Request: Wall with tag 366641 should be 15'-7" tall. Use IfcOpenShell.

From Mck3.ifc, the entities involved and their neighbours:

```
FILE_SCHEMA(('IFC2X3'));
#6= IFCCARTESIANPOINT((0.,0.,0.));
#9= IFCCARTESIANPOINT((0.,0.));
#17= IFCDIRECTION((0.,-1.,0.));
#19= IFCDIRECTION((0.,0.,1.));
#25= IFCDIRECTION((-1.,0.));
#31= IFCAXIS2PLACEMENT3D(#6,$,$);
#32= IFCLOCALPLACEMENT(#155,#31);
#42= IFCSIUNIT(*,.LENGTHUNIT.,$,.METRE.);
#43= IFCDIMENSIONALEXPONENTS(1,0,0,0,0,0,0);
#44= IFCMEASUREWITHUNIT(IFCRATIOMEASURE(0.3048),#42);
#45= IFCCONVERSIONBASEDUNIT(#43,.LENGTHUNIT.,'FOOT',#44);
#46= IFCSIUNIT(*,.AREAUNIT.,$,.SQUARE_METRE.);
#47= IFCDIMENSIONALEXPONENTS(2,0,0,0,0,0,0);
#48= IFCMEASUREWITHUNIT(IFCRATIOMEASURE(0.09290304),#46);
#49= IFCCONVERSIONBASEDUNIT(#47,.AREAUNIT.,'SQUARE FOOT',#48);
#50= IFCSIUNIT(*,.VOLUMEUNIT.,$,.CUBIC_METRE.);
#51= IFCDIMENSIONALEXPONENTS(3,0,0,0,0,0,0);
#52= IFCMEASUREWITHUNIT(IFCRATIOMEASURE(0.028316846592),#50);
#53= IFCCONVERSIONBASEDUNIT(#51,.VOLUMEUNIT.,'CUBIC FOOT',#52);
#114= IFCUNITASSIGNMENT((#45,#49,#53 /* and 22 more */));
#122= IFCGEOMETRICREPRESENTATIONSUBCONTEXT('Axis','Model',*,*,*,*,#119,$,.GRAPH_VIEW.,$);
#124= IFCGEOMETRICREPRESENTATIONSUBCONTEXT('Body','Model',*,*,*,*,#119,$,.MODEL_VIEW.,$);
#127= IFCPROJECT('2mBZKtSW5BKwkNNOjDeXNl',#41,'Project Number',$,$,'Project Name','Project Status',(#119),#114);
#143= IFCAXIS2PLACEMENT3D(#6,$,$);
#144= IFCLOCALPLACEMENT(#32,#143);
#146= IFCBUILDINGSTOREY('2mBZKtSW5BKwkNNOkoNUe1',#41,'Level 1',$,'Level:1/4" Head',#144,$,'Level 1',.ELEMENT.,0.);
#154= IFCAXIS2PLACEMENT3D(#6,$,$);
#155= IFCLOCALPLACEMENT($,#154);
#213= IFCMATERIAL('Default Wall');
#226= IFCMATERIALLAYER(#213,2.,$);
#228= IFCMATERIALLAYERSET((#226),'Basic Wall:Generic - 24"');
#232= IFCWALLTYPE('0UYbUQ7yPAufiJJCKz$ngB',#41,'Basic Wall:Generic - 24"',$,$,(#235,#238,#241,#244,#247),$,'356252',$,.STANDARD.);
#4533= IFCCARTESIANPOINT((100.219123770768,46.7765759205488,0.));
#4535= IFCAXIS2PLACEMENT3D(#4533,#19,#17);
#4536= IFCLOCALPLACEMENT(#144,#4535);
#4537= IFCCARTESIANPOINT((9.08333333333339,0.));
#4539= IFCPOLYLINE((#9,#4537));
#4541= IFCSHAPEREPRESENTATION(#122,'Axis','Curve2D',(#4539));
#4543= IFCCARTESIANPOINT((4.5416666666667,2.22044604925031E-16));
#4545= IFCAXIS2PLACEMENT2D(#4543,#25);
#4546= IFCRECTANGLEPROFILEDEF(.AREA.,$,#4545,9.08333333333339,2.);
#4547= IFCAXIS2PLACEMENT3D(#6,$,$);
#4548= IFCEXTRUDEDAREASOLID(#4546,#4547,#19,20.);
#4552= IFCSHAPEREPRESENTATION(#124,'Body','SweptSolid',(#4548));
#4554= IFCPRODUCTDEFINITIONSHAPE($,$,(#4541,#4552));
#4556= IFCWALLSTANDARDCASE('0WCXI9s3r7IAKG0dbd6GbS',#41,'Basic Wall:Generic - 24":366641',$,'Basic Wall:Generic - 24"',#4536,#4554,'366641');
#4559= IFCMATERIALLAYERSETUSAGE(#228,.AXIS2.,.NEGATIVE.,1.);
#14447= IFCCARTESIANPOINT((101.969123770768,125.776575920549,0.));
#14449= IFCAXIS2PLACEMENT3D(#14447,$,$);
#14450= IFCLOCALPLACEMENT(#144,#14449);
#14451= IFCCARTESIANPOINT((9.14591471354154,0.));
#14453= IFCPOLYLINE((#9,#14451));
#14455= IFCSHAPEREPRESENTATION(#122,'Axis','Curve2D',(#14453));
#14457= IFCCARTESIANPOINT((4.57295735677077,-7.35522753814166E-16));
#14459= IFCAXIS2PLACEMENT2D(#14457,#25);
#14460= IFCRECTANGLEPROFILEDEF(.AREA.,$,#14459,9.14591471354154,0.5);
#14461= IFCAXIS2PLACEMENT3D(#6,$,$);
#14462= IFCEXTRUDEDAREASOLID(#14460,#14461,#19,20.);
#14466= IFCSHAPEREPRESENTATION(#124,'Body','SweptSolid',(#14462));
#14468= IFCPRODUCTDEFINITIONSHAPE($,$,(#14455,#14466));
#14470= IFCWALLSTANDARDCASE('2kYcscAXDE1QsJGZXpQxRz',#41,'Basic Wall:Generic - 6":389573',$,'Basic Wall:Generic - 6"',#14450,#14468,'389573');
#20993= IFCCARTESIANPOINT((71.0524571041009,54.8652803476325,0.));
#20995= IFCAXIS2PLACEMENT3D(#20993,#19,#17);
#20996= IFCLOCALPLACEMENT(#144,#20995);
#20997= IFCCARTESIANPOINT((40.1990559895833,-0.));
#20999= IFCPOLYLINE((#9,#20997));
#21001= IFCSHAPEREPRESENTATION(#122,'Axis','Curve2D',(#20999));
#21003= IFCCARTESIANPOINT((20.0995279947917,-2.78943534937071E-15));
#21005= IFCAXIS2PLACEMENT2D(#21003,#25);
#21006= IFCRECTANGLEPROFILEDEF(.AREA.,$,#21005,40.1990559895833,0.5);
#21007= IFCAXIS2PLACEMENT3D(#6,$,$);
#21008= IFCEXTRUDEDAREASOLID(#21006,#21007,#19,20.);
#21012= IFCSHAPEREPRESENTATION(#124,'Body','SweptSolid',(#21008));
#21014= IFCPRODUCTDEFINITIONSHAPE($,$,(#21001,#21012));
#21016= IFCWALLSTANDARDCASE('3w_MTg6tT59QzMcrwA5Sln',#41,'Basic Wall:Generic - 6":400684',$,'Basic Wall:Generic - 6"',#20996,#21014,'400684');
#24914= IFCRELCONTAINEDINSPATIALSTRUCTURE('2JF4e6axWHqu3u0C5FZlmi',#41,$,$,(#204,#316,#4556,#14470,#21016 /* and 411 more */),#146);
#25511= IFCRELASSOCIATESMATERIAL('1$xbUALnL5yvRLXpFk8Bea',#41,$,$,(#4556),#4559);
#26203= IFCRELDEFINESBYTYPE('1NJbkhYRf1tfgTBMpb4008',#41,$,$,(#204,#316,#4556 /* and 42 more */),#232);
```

```python
import ifcopenshell
import ifcopenshell.geom
import ifcopenshell.util.representation
import ifcopenshell.util.shape
import ifcopenshell.util.unit

model = ifcopenshell.open("Mck3.ifc")
unit_scale = ifcopenshell.util.unit.calculate_unit_scale(model)
settings = ifcopenshell.geom.settings()


def volume(element):
    """Net volume in cubic metres, openings subtracted."""
    shape = ifcopenshell.geom.create_shape(settings, element)
    return ifcopenshell.util.shape.get_volume(shape.geometry)


wall = model.by_guid("0WCXI9s3r7IAKG0dbd6GbS")
before = volume(wall)

body = ifcopenshell.util.representation.get_representation(wall, "Model", "Body")
solid = body.Items[0]
old_height = solid.Depth
solid.Depth = 187 * 0.0254 / unit_scale
after = volume(wall)

print(f"height {old_height:g} -> {solid.Depth:g}, volume {before:.3f} -> {after:.3f} m3")

model.write("Mck3_updated.ifc")
```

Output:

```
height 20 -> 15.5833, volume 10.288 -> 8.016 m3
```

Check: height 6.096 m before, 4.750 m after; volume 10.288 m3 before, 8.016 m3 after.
